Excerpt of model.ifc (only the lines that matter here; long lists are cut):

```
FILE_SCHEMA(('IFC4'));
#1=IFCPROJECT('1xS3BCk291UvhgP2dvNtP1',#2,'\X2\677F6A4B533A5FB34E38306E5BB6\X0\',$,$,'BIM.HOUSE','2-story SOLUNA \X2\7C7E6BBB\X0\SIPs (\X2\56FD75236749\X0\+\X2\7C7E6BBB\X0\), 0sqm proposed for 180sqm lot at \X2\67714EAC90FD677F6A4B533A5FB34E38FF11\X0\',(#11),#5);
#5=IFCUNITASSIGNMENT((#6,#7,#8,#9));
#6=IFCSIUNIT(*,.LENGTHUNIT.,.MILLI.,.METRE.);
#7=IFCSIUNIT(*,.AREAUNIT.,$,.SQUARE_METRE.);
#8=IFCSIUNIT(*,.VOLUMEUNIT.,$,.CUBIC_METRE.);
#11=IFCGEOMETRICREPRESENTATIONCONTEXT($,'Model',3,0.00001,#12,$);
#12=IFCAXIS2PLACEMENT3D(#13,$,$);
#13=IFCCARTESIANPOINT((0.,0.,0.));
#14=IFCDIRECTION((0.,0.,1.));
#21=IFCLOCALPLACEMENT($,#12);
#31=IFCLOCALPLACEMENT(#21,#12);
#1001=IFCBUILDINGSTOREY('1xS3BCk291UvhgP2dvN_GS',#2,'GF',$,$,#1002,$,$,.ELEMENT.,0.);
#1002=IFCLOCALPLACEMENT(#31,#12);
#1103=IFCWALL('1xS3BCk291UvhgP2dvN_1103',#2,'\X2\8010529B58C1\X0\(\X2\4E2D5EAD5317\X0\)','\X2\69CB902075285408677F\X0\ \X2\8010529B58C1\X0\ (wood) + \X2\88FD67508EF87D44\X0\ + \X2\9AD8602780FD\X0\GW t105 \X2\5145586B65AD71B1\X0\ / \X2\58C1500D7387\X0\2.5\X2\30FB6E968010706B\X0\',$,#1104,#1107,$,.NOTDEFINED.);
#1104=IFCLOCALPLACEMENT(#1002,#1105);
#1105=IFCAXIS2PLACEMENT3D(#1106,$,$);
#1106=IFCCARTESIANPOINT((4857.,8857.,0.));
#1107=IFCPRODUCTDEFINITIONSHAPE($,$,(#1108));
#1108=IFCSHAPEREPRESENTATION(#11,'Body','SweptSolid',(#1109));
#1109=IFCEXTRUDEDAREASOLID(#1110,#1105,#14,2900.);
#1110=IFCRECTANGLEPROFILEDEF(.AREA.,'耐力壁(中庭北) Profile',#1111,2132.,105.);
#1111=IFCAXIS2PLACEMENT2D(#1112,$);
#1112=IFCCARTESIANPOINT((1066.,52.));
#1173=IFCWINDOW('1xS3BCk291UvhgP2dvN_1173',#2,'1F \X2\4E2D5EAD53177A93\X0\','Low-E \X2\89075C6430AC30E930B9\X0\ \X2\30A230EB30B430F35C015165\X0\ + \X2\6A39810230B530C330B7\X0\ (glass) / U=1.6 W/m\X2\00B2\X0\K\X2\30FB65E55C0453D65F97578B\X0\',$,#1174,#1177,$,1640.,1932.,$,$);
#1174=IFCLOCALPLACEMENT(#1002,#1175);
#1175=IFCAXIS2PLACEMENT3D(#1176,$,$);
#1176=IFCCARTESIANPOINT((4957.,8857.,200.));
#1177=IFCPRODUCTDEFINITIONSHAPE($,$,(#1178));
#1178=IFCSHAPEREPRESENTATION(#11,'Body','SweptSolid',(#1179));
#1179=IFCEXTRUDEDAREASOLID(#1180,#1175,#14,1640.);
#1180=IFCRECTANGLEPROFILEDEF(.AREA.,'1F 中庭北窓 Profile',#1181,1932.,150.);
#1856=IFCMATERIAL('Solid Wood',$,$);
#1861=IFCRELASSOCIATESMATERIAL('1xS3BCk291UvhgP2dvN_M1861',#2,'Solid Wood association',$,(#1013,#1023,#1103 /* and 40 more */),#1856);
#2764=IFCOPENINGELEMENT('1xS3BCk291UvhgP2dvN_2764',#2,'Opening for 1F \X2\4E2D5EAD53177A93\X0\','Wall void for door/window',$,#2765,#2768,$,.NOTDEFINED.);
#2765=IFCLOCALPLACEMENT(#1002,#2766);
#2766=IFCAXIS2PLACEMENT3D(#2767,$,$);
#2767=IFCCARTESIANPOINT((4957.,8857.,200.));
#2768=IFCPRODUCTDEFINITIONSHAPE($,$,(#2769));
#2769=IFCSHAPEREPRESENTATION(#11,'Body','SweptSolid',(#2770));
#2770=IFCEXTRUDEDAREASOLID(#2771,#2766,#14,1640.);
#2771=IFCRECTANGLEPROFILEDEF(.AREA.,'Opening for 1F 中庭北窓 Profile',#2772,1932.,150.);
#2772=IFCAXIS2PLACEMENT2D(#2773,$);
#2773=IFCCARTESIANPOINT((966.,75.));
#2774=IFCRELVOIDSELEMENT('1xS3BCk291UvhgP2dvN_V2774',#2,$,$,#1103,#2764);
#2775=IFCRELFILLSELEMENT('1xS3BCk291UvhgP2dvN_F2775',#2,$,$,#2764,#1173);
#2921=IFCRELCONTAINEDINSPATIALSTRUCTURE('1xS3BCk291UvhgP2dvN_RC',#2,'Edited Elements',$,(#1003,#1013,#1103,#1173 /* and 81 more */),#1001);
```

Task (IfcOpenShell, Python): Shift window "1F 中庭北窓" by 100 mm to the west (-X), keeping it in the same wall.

```python
import ifcopenshell
import ifcopenshell.api.geometry
import ifcopenshell.util.placement
import ifcopenshell.util.unit

model = ifcopenshell.open("model.ifc")
unit_scale = ifcopenshell.util.unit.calculate_unit_scale(model)

window = model.by_id(1173)
opening = window.FillsVoids[0].RelatingOpeningElement
wall = opening.VoidsElements[0].RelatingBuildingElement

wall_matrix = ifcopenshell.util.placement.get_local_placement(wall.ObjectPlacement)
shift = wall_matrix[:3, 0] * -0.1 / unit_scale
before = ifcopenshell.util.placement.get_local_placement(window.ObjectPlacement)[:3, 3].copy()

# The window is not placed relative to its opening, so move both.
for product in (opening, window):
    matrix = ifcopenshell.util.placement.get_local_placement(product.ObjectPlacement)
    matrix[:3, 3] += shift
    ifcopenshell.api.geometry.edit_object_placement(model, product=product, matrix=matrix, is_si=False)

after = ifcopenshell.util.placement.get_local_placement(window.ObjectPlacement)[:3, 3]
print("window moved by", (after - before).round(3) + 0.0)

model.write("model_v2.ifc")
```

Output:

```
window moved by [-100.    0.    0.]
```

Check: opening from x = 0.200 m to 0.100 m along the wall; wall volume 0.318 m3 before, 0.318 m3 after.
